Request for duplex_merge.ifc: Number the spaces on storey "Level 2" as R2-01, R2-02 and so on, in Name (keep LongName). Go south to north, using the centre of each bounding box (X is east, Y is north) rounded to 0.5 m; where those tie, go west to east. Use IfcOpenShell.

First a look at what the model holds.

```python
import ifcopenshell
import ifcopenshell.util.element
import ifcopenshell.util.placement

model = ifcopenshell.open("duplex_merge.ifc")
print(model.schema)
storey = next(s for s in model.by_type("IfcBuildingStorey") if s.Name == "Level 2")
spaces = [e for e in ifcopenshell.util.element.get_decomposition(storey) if e.is_a("IfcSpace")]
for e in sorted(spaces, key=lambda e: e.id()):
    origin = ifcopenshell.util.placement.get_local_placement(e.ObjectPlacement)[:3, 3]
    print(e.id(), e.Name, e.LongName, origin.round(2) + 0.0, sep=" | ")
```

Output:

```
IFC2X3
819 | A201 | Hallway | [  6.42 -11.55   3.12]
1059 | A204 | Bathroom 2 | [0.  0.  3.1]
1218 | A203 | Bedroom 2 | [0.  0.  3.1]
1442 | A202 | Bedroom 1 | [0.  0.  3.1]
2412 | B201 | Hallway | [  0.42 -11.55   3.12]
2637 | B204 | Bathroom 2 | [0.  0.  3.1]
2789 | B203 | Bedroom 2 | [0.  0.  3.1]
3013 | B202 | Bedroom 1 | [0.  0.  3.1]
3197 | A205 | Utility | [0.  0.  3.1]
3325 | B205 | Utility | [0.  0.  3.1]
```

```python
import ifcopenshell
import ifcopenshell.geom
import ifcopenshell.util.element
import ifcopenshell.util.shape

model = ifcopenshell.open("duplex_merge.ifc")
settings = ifcopenshell.geom.settings()
settings.set("use-world-coords", True)


def centre(element):
    shape = ifcopenshell.geom.create_shape(settings, element)
    return ifcopenshell.util.shape.get_bbox_centroid(shape.geometry)


storey = next(s for s in model.by_type("IfcBuildingStorey") if s.Name == "Level 2")
spaces = [e for e in ifcopenshell.util.element.get_decomposition(storey) if e.is_a("IfcSpace")]

# Insertion points can sit at a corner or the storey origin, so sort by the geometry (in metres).
centres = {e: centre(e) for e in spaces}
spaces.sort(key=lambda e: (round(centres[e][1] / 0.5), centres[e][0]))

for i, e in enumerate(spaces, start=1):
    number = f"R2-{i:02d}"
    e.Name = number
    print(e.id(), number)

model.write("duplex_merge_edited.ifc")
```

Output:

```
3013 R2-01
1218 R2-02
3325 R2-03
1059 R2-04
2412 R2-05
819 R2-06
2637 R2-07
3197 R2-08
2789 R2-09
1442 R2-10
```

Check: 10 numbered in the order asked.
